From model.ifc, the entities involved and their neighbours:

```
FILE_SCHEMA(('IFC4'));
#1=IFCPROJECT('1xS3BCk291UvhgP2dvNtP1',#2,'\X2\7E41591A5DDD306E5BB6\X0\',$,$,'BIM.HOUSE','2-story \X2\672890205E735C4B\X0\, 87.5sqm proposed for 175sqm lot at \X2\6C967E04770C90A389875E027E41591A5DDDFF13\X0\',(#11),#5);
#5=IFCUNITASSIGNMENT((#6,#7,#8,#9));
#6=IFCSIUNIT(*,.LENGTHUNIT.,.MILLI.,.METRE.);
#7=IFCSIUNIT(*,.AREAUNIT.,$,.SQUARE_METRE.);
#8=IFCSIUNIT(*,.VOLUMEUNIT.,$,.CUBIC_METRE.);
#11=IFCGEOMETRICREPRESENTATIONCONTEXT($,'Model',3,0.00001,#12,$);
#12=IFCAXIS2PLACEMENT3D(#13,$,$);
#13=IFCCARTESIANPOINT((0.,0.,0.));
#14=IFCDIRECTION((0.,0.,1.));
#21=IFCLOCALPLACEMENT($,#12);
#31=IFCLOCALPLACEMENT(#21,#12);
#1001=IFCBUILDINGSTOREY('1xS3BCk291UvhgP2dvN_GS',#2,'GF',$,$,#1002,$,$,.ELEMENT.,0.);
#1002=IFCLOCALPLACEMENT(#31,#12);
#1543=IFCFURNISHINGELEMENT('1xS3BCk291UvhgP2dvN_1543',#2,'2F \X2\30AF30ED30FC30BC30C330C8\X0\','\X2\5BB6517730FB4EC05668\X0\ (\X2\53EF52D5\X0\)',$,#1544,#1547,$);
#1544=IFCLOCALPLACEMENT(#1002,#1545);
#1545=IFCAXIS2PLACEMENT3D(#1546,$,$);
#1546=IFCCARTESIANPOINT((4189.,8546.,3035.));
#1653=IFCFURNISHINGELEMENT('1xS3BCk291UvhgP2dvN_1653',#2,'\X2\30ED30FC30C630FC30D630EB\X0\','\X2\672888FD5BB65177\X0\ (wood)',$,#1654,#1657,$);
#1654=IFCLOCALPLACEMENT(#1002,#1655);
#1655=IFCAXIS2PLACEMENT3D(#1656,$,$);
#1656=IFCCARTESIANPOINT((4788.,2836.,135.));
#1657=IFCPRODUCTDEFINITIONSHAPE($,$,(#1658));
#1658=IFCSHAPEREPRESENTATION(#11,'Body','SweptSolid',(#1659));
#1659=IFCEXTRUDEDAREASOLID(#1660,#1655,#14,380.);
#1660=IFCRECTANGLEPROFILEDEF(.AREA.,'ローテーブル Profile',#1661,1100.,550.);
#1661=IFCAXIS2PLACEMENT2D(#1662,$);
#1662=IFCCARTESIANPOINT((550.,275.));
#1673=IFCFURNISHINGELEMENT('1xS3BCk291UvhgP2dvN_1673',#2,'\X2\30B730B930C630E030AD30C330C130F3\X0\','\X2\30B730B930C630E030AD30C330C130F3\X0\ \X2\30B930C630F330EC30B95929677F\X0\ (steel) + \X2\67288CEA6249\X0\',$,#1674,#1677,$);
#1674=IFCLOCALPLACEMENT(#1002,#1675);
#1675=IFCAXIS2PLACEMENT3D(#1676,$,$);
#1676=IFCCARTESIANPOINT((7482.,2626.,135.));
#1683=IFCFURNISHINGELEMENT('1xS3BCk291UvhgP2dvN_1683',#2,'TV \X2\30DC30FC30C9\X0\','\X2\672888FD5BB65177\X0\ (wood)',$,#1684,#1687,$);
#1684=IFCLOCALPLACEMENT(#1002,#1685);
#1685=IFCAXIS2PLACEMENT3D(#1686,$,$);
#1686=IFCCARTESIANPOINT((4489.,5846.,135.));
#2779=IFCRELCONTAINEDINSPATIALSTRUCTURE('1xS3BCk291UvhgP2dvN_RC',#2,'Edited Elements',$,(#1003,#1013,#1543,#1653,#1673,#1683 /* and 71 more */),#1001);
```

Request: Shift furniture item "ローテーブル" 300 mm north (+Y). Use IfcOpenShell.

```python
import ifcopenshell
import ifcopenshell.api.geometry
import ifcopenshell.util.placement

model = ifcopenshell.open("model.ifc")

item = model.by_guid("1xS3BCk291UvhgP2dvN_1653")
matrix = ifcopenshell.util.placement.get_local_placement(item.ObjectPlacement)
matrix[1, 3] += 300.0
ifcopenshell.api.geometry.edit_object_placement(model, product=item, matrix=matrix, is_si=False)

print(ifcopenshell.util.placement.get_local_placement(item.ObjectPlacement).round(3) + 0.0)

model.write("model_v2.ifc")
```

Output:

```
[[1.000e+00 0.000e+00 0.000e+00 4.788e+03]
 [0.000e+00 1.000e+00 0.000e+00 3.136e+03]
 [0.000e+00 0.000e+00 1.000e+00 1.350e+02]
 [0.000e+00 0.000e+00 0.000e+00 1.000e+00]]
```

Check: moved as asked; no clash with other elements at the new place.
